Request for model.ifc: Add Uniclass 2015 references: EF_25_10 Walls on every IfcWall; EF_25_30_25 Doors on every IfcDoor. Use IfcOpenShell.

First a look at what the model holds.

```python
import ifcopenshell

model = ifcopenshell.open("model.ifc")
print(model.schema)
print("classifications:", [c.Name for c in model.by_type("IfcClassification")])
for ifc_class in ("IfcDoor", "IfcRoof", "IfcStair", "IfcWall", "IfcWindow"):
    print(ifc_class, len(model.by_type(ifc_class)))
```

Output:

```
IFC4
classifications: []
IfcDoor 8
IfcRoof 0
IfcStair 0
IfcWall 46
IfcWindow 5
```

```python
import ifcopenshell
import ifcopenshell.api.classification

model = ifcopenshell.open("model.ifc")

system = ifcopenshell.api.classification.add_classification(model, classification="Uniclass 2015")

codes = {
    "IfcWall": ("EF_25_10", "Walls"),
    "IfcDoor": ("EF_25_30_25", "Doors"),
}
for ifc_class, (code, name) in codes.items():
    products = model.by_type(ifc_class)
    ifcopenshell.api.classification.add_reference(
        model, products=products, classification=system, identification=code, name=name
    )
    print(code, len(products))

model.write("model-out.ifc")
```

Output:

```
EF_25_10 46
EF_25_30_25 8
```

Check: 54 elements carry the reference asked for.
